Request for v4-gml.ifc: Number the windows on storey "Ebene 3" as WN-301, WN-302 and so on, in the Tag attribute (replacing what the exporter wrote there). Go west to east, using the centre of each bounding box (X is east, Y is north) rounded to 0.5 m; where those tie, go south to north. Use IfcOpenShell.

First a look at what the model holds.

```python
import ifcopenshell
import ifcopenshell.util.element
import ifcopenshell.util.placement

model = ifcopenshell.open("v4-gml.ifc")
print(model.schema)
storey = next(s for s in model.by_type("IfcBuildingStorey") if s.Name == "Ebene 3")
windows = [e for e in ifcopenshell.util.element.get_decomposition(storey) if e.is_a("IfcWindow")]
for e in sorted(windows, key=lambda e: e.id()):
    origin = ifcopenshell.util.placement.get_local_placement(e.ObjectPlacement)[:3, 3]
    print(e.id(), e.Tag, e.Name, origin.round(2) + 0.0, sep=" | ")
```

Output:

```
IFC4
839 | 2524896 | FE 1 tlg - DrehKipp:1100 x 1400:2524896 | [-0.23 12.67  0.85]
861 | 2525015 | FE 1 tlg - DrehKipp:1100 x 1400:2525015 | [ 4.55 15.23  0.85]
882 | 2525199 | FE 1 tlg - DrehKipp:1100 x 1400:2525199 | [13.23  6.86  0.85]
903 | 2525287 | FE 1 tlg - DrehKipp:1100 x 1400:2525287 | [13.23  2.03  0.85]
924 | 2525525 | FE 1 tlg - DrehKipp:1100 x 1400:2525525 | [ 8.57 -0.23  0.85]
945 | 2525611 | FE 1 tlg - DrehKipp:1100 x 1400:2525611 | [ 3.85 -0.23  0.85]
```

```python
import ifcopenshell
import ifcopenshell.geom
import ifcopenshell.util.element
import ifcopenshell.util.shape

model = ifcopenshell.open("v4-gml.ifc")
settings = ifcopenshell.geom.settings()
settings.set("use-world-coords", True)


def centre(element):
    shape = ifcopenshell.geom.create_shape(settings, element)
    return ifcopenshell.util.shape.get_bbox_centroid(shape.geometry)


storey = next(s for s in model.by_type("IfcBuildingStorey") if s.Name == "Ebene 3")
windows = [e for e in ifcopenshell.util.element.get_decomposition(storey) if e.is_a("IfcWindow")]

# Insertion points can sit at a corner or the storey origin, so sort by the geometry (in metres).
centres = {e: centre(e) for e in windows}
windows.sort(key=lambda e: (round(centres[e][0] / 0.5), centres[e][1]))

for i, e in enumerate(windows, start=1):
    number = f"WN-3{i:02d}"
    e.Tag = number
    print(e.id(), number)

model.write("v4-gml_v2.ifc")
```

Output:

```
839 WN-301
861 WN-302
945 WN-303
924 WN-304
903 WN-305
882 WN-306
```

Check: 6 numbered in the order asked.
